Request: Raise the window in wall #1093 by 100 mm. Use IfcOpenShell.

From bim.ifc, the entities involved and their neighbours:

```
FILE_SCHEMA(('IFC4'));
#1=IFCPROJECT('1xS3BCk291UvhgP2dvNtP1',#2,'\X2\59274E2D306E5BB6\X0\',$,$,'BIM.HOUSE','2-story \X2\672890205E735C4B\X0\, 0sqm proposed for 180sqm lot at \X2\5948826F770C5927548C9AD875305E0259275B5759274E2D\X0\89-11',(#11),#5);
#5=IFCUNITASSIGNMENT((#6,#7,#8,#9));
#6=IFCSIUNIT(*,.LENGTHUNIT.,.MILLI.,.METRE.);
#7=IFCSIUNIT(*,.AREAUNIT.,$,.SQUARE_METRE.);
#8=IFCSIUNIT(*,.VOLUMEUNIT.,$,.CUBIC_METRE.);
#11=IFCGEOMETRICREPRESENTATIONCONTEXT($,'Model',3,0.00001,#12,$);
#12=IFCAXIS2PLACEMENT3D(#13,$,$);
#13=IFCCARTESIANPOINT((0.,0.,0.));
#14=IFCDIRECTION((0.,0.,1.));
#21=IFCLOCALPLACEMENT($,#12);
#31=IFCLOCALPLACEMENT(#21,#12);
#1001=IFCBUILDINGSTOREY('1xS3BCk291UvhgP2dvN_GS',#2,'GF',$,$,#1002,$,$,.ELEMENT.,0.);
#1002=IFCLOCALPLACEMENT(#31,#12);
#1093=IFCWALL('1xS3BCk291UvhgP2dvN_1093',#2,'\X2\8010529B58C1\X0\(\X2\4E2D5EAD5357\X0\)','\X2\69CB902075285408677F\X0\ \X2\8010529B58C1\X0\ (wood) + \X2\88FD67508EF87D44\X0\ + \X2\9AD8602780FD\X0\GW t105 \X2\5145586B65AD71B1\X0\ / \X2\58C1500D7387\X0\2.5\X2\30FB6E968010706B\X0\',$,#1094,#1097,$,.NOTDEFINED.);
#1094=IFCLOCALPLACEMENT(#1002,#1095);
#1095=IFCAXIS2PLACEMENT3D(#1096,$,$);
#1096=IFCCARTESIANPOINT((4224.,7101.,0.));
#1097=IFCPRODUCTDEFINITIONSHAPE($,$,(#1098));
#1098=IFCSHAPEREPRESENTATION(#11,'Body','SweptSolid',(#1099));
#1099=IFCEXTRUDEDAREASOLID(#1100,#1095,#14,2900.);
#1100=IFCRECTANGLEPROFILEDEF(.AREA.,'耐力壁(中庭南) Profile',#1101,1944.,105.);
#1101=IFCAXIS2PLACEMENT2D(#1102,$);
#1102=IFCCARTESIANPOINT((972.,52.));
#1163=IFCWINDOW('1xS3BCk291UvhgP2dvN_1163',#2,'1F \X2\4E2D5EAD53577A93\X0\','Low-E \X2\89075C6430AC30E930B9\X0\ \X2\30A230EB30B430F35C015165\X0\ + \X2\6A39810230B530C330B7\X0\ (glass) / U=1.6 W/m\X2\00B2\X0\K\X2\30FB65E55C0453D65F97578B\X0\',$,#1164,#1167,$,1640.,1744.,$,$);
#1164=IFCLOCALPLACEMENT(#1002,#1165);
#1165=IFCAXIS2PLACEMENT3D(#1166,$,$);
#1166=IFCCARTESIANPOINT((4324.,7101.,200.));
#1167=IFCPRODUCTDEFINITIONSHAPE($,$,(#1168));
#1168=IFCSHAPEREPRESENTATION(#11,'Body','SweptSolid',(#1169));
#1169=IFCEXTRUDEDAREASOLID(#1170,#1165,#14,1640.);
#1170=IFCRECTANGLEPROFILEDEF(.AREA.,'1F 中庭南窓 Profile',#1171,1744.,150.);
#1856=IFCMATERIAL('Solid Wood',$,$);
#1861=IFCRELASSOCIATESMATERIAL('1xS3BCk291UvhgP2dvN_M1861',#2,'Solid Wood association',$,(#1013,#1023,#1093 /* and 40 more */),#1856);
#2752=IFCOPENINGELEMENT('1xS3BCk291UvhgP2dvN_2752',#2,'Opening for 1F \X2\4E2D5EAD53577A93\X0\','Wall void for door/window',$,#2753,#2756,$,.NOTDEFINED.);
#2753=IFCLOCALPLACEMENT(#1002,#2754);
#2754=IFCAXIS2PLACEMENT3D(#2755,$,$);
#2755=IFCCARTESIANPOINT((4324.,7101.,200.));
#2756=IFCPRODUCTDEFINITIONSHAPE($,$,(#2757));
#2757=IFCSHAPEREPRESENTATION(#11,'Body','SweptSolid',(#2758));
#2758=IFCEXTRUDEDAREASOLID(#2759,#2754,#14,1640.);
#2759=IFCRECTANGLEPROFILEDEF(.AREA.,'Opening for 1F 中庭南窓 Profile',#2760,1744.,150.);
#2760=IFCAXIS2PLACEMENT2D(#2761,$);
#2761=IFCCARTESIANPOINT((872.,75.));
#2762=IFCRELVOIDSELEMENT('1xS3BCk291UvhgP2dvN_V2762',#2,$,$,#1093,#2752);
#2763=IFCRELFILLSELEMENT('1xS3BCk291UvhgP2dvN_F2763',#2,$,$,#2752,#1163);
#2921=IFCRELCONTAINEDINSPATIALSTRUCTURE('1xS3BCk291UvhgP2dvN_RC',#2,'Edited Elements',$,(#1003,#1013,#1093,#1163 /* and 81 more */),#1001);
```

```python
import numpy as np
import ifcopenshell
import ifcopenshell.api.geometry
import ifcopenshell.util.placement
import ifcopenshell.util.unit

model = ifcopenshell.open("bim.ifc")
unit_scale = ifcopenshell.util.unit.calculate_unit_scale(model)

window = model.by_guid("1xS3BCk291UvhgP2dvN_1163")
opening = window.FillsVoids[0].RelatingOpeningElement
dz = 100.0

shift = np.array([0.0, 0.0, dz])
# The window is not placed relative to its opening, so move both.
for product in (opening, window):
    matrix = ifcopenshell.util.placement.get_local_placement(product.ObjectPlacement)
    matrix[:3, 3] += shift
    ifcopenshell.api.geometry.edit_object_placement(model, product=product, matrix=matrix, is_si=False)

print(f"moved by {dz * unit_scale:+.3f} m")

model.write("bim_v2.ifc")
```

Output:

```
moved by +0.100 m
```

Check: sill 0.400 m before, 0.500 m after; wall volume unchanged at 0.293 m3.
